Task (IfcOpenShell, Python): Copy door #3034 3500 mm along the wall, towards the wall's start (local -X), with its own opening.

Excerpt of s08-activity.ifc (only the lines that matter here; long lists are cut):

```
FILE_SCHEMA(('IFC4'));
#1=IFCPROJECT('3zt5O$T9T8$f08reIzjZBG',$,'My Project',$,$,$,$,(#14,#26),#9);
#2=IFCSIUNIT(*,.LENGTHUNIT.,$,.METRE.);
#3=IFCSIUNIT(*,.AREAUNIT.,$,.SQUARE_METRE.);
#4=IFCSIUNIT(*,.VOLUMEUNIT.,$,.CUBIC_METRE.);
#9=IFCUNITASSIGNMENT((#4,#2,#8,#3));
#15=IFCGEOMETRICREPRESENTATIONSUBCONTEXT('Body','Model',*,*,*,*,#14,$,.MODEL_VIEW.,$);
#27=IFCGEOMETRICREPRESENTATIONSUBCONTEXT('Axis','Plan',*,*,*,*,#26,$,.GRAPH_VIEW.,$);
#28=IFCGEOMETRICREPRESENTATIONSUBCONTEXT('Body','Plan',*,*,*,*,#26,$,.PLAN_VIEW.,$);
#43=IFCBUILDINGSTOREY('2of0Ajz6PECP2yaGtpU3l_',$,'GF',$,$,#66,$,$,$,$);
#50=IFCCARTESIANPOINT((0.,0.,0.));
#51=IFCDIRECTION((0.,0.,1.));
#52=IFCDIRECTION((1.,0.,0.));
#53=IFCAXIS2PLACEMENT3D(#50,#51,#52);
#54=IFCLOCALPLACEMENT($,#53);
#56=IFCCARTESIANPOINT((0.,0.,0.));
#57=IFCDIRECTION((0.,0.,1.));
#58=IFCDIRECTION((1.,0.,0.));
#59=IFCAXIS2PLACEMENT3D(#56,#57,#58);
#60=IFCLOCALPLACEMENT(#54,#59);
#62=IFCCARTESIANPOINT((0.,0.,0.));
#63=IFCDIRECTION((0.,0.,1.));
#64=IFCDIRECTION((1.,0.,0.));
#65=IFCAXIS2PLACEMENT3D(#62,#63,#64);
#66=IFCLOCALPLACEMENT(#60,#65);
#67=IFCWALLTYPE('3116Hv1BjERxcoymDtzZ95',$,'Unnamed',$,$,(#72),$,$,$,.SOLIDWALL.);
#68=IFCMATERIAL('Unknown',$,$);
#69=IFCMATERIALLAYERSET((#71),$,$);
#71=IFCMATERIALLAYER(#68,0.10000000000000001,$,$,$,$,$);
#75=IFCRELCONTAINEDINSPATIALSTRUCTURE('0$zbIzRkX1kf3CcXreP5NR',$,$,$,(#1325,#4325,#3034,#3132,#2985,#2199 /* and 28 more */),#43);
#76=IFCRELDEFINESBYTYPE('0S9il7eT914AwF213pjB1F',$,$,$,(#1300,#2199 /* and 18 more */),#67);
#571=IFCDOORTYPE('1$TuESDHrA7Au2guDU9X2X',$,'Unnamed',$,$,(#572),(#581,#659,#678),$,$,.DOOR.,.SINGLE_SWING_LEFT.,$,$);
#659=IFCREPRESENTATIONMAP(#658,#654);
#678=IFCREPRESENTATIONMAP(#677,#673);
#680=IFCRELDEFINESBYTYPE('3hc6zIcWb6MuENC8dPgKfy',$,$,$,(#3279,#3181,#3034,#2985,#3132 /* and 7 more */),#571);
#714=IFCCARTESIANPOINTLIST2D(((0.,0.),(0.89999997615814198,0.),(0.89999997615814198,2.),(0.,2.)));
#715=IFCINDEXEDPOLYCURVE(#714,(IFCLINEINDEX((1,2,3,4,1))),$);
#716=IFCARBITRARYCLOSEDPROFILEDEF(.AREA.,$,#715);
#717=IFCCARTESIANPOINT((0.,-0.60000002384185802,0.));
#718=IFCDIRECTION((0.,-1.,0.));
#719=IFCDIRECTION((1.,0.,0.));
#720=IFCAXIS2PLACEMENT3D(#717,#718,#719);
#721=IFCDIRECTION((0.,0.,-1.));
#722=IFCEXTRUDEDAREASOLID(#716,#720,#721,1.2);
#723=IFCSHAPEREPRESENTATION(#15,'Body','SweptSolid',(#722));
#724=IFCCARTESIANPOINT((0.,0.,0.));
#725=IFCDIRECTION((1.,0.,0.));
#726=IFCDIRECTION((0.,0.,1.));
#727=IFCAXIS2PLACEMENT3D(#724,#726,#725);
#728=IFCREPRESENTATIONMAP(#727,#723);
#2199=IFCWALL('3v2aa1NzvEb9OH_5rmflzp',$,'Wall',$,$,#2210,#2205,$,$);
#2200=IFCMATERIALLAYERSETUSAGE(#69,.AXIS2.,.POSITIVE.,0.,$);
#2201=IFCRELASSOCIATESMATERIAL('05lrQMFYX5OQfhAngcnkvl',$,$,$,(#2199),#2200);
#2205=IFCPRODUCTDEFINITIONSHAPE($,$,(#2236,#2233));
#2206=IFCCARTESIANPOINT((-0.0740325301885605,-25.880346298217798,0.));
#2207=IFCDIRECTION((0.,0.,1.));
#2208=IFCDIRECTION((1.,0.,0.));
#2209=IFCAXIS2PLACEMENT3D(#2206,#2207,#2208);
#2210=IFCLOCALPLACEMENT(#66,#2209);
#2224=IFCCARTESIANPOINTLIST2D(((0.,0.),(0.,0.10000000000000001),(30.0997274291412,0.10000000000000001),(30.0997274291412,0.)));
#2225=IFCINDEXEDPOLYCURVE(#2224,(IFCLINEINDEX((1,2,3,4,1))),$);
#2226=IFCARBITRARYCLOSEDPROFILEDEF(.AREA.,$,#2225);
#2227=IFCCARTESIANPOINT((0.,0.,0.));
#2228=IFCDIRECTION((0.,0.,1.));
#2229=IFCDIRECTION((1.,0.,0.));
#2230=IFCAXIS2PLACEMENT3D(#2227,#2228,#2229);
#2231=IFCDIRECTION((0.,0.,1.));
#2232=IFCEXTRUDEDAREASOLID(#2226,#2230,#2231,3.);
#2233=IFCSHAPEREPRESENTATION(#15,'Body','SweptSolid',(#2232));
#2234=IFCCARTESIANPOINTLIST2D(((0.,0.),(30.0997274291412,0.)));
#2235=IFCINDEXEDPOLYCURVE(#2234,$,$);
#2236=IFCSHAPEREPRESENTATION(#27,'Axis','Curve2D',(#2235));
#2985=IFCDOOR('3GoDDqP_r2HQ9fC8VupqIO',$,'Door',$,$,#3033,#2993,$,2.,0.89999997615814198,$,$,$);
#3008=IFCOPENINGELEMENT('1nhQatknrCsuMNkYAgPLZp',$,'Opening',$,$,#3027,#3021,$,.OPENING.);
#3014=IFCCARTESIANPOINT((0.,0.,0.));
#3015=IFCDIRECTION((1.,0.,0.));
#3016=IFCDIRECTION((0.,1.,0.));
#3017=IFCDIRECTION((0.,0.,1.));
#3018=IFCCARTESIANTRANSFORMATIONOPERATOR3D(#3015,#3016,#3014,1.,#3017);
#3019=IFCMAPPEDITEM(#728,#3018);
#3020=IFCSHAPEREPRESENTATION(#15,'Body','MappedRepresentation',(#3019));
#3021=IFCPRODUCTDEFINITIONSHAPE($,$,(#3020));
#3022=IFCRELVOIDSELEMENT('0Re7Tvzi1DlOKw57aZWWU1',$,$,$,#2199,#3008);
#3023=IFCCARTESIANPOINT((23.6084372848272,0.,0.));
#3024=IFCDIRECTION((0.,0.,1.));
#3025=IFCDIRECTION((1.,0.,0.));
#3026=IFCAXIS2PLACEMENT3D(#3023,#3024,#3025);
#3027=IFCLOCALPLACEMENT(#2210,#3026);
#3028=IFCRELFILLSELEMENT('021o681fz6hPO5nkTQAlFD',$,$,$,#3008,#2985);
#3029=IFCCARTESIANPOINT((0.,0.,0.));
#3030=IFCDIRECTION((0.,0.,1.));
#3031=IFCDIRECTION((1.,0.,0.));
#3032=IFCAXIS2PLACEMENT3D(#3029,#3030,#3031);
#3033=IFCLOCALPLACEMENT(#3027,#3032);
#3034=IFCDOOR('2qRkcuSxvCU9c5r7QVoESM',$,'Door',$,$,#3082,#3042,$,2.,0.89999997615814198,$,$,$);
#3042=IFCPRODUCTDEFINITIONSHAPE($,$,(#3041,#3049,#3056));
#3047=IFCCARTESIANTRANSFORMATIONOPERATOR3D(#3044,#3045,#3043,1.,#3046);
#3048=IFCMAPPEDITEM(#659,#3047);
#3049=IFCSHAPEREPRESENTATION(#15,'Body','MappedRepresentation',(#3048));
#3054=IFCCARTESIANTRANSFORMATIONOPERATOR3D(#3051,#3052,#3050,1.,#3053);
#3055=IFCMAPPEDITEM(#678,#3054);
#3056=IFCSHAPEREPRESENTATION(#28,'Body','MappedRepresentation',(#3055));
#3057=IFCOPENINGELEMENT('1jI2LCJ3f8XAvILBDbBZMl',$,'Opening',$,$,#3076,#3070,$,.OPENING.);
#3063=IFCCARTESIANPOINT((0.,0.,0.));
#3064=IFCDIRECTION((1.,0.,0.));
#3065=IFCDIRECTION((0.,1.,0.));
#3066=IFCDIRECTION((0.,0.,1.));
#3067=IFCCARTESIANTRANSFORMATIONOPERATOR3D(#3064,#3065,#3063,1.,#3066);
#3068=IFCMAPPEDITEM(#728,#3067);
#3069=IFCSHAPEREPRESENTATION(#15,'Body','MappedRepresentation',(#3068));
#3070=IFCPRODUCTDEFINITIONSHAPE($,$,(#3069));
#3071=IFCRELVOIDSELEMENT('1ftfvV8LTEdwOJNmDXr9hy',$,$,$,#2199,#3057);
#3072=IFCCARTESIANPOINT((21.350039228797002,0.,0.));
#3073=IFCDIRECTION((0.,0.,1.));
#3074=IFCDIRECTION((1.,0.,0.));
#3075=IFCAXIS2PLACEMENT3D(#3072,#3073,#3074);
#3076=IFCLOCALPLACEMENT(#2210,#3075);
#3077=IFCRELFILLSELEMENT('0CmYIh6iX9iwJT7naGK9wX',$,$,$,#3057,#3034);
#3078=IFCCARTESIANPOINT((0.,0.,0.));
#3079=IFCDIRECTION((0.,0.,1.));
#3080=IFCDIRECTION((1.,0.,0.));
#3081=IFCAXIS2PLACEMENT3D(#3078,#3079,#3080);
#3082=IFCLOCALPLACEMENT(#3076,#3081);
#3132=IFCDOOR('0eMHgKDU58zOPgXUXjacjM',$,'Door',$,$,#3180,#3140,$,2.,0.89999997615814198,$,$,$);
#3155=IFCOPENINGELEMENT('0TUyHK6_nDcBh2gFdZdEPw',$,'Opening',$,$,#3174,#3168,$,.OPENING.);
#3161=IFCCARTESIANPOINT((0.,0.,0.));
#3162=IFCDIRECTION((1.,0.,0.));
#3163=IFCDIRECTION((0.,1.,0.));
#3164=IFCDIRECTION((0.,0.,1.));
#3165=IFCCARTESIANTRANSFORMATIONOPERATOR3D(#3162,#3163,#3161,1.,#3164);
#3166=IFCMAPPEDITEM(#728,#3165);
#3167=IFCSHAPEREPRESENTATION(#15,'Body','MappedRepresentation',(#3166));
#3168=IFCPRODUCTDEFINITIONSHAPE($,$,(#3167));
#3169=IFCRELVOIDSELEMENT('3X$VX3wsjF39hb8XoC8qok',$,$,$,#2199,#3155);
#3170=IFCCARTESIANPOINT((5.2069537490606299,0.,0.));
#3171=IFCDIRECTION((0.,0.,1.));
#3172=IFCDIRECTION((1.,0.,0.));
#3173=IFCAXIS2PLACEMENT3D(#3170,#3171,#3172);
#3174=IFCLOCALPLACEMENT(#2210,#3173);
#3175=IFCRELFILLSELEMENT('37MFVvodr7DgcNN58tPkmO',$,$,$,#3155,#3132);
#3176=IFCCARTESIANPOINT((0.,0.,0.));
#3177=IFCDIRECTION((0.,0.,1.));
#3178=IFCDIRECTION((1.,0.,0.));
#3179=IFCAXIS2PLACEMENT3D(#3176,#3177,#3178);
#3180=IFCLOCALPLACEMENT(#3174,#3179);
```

```python
import ifcopenshell
import ifcopenshell.api.feature
import ifcopenshell.api.geometry
import ifcopenshell.api.root
import ifcopenshell.geom
import ifcopenshell.util.element
import ifcopenshell.util.placement
import ifcopenshell.util.shape
import ifcopenshell.util.unit

model = ifcopenshell.open("s08-activity.ifc")
unit_scale = ifcopenshell.util.unit.calculate_unit_scale(model)
settings = ifcopenshell.geom.settings()


def volume(element):
    """Net volume in cubic metres, openings subtracted."""
    shape = ifcopenshell.geom.create_shape(settings, element)
    return ifcopenshell.util.shape.get_volume(shape.geometry)


door = model.by_guid("2qRkcuSxvCU9c5r7QVoESM")
opening = door.FillsVoids[0].RelatingOpeningElement
wall = opening.VoidsElements[0].RelatingBuildingElement
before = volume(wall)
shift = ifcopenshell.util.placement.get_local_placement(wall.ObjectPlacement)[:3, 0] * -3.5 / unit_scale

# copy_class copies the void relationship, type, container and properties, but no geometry.
new_opening = ifcopenshell.api.root.copy_class(model, product=opening)
new_opening.Representation = ifcopenshell.util.element.copy_deep(
    model, opening.Representation, exclude=["IfcGeometricRepresentationContext", "IfcRepresentationMap"]
)
new_door = ifcopenshell.api.root.copy_class(model, product=door)
new_door.Representation = ifcopenshell.util.element.copy_deep(
    model, door.Representation, exclude=["IfcGeometricRepresentationContext", "IfcRepresentationMap"]
)
ifcopenshell.api.feature.add_filling(model, opening=new_opening, element=new_door)

for old, new in ((opening, new_opening), (door, new_door)):
    matrix = ifcopenshell.util.placement.get_local_placement(old.ObjectPlacement)
    matrix[:3, 3] += shift
    ifcopenshell.api.geometry.edit_object_placement(model, product=new, matrix=matrix, is_si=False)

after = volume(wall)

print(f"wall volume {before:.3f} -> {after:.3f} m3")

model.write("s08-activity-out.ifc")
```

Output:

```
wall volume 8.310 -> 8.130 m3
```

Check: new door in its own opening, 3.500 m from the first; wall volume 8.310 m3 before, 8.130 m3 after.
